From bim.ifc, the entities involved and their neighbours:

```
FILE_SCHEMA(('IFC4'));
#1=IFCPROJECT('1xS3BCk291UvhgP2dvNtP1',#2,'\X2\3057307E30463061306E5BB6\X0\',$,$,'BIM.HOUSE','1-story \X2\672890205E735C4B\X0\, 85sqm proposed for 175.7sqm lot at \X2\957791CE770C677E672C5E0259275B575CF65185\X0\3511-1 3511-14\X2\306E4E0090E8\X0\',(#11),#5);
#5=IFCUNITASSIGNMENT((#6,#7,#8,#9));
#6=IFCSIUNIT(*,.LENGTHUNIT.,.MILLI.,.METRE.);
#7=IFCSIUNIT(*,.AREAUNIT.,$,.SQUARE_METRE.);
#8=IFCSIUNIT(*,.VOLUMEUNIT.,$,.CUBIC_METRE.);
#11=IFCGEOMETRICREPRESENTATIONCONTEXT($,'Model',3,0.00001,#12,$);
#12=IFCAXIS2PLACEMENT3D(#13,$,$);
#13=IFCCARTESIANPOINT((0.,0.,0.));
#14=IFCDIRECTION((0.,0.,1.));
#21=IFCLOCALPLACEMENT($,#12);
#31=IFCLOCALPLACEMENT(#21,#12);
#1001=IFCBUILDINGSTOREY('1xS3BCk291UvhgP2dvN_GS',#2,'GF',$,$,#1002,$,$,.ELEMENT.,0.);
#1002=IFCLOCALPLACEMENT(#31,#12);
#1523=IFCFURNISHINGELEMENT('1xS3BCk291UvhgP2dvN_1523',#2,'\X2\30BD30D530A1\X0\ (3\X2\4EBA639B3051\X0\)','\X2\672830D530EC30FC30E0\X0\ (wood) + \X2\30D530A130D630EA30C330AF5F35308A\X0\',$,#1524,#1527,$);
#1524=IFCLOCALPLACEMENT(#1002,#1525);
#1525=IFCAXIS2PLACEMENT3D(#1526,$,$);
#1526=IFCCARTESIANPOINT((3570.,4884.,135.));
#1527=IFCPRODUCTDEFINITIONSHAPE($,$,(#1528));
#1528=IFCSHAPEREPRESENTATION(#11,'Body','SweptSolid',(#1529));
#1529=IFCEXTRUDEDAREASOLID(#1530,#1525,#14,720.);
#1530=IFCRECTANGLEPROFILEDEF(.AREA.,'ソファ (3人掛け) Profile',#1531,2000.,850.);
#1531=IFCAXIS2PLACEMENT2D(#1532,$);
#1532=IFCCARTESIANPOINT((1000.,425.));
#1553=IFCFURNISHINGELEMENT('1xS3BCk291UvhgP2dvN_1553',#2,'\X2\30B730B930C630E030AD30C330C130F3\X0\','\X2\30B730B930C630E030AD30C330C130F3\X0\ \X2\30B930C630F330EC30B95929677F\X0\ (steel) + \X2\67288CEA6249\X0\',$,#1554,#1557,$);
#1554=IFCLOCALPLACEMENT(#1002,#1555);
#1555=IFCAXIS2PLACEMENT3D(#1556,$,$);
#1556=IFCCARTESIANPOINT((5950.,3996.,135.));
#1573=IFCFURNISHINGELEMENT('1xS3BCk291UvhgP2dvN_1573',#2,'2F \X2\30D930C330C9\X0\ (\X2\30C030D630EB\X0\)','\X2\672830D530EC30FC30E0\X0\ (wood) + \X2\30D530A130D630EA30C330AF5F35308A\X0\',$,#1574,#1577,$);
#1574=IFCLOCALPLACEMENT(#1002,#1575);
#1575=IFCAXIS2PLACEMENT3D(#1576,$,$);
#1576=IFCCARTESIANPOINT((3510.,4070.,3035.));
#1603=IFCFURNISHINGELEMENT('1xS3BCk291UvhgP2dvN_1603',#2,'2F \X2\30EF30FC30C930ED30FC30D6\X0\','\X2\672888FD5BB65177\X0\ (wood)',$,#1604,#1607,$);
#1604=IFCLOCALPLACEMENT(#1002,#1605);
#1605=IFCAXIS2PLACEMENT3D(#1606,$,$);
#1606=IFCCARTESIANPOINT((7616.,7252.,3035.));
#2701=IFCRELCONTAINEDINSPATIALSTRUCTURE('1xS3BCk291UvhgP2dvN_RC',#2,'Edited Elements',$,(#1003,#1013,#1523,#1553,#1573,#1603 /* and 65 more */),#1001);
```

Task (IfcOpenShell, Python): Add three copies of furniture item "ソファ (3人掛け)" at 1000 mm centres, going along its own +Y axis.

```python
import ifcopenshell
import ifcopenshell.api.geometry
import ifcopenshell.api.root
import ifcopenshell.util.element
import ifcopenshell.util.placement
import ifcopenshell.util.unit

model = ifcopenshell.open("bim.ifc")
unit_scale = ifcopenshell.util.unit.calculate_unit_scale(model)


def reuse_history(source, copy):
    """copy_class also copies each property set's owner history, people and application; keep the originals."""
    for rel in copy.IsDefinedBy:
        if rel.is_a("IfcRelDefinesByProperties") and (history := rel.RelatingPropertyDefinition.OwnerHistory):
            rel.RelatingPropertyDefinition.OwnerHistory = source.OwnerHistory
            ifcopenshell.util.element.remove_deep2(model, history)


source = model.by_guid("1xS3BCk291UvhgP2dvN_1523")
base = ifcopenshell.util.placement.get_local_placement(source.ObjectPlacement)
step = base[:3, 1] * 1 / unit_scale

for i in range(1, 4):
    copy = ifcopenshell.api.root.copy_class(model, product=source)
    copy.Representation = ifcopenshell.util.element.copy_deep(
        model, source.Representation, exclude=["IfcGeometricRepresentationContext", "IfcRepresentationMap"]
    )
    reuse_history(source, copy)
    matrix = base.copy()
    matrix[:3, 3] += i * step
    print("added at", matrix[:3, 3].round(3) + 0.0)
    ifcopenshell.api.geometry.edit_object_placement(model, product=copy, matrix=matrix, is_si=False)

model.write("bim_v2.ifc")
```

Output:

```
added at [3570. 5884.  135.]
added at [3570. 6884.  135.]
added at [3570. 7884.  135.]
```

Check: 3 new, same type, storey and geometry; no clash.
